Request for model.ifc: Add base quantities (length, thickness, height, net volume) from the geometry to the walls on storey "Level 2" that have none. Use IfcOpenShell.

First a look at what the model holds.

```python
import ifcopenshell
import ifcopenshell.util.element
import ifcopenshell.util.unit

model = ifcopenshell.open("model.ifc")
print(model.schema)
for unit_type in ("LENGTHUNIT", "AREAUNIT", "VOLUMEUNIT"):
    print(unit_type, ifcopenshell.util.unit.calculate_unit_scale(model, unit_type))
storey = next(s for s in model.by_type("IfcBuildingStorey") if s.Name == "Level 2")
walls = [e for e in ifcopenshell.util.element.get_decomposition(storey) if e.is_a("IfcWall")]
for e in sorted(walls, key=lambda e: e.id()):
    print(e.id(), e.is_a(), e.Name, list(ifcopenshell.util.element.get_psets(e, qtos_only=True)), sep=" | ")
```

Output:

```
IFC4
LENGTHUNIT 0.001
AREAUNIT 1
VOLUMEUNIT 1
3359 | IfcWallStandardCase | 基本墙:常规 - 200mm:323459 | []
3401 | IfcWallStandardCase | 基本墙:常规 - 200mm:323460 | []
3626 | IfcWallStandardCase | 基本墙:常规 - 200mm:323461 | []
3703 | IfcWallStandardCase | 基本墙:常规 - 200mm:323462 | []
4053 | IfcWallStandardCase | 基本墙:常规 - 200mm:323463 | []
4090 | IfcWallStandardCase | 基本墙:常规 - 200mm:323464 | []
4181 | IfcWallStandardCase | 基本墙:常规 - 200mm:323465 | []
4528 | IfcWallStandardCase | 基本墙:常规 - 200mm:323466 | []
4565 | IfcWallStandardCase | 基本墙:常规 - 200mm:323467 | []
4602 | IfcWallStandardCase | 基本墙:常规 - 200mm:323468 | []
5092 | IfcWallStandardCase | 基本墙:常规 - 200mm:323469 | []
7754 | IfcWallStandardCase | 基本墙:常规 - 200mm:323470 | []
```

```python
import ifcopenshell
import ifcopenshell.api.pset
import ifcopenshell.geom
import ifcopenshell.util.element
import ifcopenshell.util.shape
import ifcopenshell.util.unit

model = ifcopenshell.open("model.ifc")
unit_scale = ifcopenshell.util.unit.calculate_unit_scale(model)
volume_scale = ifcopenshell.util.unit.calculate_unit_scale(model, "VOLUMEUNIT")
settings = ifcopenshell.geom.settings()

storey = next(s for s in model.by_type("IfcBuildingStorey") if s.Name == "Level 2")
walls = [e for e in ifcopenshell.util.element.get_decomposition(storey) if e.is_a("IfcWall")]

for e in sorted(walls, key=lambda e: e.id()):
    if ifcopenshell.util.element.get_psets(e, qtos_only=True, should_inherit=False):
        continue
    # Geometry comes back in metres, in the element's own axes.
    shape = ifcopenshell.geom.create_shape(settings, e)
    values = {
        "Length": ifcopenshell.util.shape.get_x(shape.geometry) / unit_scale,
        "Width": ifcopenshell.util.shape.get_y(shape.geometry) / unit_scale,
        "Height": ifcopenshell.util.shape.get_z(shape.geometry) / unit_scale,
        "NetVolume": ifcopenshell.util.shape.get_volume(shape.geometry) / volume_scale,
    }
    qto = ifcopenshell.api.pset.add_qto(model, product=e, name="Qto_WallBaseQuantities")
    ifcopenshell.api.pset.edit_qto(model, qto=qto, properties=values)
    print(e.id(), {k: round(v, 3) for k, v in values.items()})

model.write("model-out.ifc")
```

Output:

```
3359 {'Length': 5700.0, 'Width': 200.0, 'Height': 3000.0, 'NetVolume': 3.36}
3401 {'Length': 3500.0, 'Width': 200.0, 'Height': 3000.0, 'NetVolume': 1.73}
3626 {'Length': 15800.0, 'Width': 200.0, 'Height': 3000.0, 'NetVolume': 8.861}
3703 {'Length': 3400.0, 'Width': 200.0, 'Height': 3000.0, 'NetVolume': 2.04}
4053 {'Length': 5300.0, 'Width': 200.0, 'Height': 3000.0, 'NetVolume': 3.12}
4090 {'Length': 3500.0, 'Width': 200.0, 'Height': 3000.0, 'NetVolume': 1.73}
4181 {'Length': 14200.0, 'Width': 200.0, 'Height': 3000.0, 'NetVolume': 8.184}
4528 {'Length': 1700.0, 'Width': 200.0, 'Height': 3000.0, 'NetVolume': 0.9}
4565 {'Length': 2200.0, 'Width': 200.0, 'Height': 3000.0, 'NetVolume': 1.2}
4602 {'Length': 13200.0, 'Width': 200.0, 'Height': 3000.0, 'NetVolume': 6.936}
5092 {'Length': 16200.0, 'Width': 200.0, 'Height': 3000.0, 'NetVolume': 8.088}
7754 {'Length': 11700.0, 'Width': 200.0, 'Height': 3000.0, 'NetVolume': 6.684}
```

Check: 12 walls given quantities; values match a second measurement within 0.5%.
